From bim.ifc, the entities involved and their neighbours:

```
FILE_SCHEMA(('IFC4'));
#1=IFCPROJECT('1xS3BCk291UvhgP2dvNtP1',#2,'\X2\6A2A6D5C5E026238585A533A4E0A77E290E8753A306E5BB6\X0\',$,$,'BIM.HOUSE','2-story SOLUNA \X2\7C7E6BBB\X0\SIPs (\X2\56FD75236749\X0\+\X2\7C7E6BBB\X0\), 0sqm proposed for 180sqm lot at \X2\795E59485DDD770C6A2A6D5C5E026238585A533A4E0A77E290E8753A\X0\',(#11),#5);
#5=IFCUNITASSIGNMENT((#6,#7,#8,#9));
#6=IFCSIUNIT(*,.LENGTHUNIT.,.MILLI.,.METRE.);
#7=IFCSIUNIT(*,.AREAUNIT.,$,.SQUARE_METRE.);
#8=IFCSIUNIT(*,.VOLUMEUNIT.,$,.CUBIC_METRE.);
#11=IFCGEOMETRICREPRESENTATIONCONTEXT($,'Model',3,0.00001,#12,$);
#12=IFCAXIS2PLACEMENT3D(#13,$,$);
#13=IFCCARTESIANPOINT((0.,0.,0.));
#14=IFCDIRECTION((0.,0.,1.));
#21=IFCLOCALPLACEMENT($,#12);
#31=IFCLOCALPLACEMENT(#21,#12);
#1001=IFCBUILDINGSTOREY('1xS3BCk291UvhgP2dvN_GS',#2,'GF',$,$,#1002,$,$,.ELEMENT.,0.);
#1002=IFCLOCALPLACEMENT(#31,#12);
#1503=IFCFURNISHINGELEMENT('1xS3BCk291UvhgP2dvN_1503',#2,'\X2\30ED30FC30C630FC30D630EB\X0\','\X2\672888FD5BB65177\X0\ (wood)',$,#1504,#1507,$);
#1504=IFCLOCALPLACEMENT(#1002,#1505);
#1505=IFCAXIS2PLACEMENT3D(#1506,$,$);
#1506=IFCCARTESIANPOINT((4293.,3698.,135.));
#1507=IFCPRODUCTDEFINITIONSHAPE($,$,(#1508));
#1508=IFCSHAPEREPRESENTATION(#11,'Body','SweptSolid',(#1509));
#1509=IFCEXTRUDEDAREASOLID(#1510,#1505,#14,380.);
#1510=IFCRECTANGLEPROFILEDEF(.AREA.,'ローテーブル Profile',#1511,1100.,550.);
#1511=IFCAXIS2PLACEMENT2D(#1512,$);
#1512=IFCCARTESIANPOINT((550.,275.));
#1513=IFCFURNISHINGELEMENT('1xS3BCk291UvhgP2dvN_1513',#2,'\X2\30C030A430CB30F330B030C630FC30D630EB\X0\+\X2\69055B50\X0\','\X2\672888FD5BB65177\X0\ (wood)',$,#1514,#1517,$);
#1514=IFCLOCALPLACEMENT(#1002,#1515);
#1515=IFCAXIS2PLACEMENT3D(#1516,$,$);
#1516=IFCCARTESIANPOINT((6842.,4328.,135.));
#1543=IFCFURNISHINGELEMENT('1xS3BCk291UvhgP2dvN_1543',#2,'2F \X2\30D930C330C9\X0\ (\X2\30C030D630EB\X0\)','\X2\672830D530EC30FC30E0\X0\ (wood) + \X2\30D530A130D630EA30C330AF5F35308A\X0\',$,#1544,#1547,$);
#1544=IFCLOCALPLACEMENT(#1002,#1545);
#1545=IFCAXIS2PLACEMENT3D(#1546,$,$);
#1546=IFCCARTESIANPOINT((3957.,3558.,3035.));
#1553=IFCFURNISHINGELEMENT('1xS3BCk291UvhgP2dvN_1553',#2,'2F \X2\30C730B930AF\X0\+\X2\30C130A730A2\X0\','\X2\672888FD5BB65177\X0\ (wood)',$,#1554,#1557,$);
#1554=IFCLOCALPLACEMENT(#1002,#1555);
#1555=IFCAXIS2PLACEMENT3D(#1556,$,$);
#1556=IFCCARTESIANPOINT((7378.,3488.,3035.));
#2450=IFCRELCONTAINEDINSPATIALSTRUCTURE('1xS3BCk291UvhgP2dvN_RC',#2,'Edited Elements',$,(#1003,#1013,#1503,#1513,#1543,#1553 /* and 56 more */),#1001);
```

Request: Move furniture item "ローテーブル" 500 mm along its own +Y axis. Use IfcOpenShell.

```python
import ifcopenshell
import ifcopenshell.api.geometry
import ifcopenshell.util.placement
import ifcopenshell.util.unit

model = ifcopenshell.open("bim.ifc")
unit_scale = ifcopenshell.util.unit.calculate_unit_scale(model)

item = model.by_guid("1xS3BCk291UvhgP2dvN_1503")
matrix = ifcopenshell.util.placement.get_local_placement(item.ObjectPlacement)
matrix[:3, 3] += matrix[:3, 1] * 0.5 / unit_scale
ifcopenshell.api.geometry.edit_object_placement(model, product=item, matrix=matrix, is_si=False)

print(ifcopenshell.util.placement.get_local_placement(item.ObjectPlacement).round(3) + 0.0)

model.write("bim_updated.ifc")
```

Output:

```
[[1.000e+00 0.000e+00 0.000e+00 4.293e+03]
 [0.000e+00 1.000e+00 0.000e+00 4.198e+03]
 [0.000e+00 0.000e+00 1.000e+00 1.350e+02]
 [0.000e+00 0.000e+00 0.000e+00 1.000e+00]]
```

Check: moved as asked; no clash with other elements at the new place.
